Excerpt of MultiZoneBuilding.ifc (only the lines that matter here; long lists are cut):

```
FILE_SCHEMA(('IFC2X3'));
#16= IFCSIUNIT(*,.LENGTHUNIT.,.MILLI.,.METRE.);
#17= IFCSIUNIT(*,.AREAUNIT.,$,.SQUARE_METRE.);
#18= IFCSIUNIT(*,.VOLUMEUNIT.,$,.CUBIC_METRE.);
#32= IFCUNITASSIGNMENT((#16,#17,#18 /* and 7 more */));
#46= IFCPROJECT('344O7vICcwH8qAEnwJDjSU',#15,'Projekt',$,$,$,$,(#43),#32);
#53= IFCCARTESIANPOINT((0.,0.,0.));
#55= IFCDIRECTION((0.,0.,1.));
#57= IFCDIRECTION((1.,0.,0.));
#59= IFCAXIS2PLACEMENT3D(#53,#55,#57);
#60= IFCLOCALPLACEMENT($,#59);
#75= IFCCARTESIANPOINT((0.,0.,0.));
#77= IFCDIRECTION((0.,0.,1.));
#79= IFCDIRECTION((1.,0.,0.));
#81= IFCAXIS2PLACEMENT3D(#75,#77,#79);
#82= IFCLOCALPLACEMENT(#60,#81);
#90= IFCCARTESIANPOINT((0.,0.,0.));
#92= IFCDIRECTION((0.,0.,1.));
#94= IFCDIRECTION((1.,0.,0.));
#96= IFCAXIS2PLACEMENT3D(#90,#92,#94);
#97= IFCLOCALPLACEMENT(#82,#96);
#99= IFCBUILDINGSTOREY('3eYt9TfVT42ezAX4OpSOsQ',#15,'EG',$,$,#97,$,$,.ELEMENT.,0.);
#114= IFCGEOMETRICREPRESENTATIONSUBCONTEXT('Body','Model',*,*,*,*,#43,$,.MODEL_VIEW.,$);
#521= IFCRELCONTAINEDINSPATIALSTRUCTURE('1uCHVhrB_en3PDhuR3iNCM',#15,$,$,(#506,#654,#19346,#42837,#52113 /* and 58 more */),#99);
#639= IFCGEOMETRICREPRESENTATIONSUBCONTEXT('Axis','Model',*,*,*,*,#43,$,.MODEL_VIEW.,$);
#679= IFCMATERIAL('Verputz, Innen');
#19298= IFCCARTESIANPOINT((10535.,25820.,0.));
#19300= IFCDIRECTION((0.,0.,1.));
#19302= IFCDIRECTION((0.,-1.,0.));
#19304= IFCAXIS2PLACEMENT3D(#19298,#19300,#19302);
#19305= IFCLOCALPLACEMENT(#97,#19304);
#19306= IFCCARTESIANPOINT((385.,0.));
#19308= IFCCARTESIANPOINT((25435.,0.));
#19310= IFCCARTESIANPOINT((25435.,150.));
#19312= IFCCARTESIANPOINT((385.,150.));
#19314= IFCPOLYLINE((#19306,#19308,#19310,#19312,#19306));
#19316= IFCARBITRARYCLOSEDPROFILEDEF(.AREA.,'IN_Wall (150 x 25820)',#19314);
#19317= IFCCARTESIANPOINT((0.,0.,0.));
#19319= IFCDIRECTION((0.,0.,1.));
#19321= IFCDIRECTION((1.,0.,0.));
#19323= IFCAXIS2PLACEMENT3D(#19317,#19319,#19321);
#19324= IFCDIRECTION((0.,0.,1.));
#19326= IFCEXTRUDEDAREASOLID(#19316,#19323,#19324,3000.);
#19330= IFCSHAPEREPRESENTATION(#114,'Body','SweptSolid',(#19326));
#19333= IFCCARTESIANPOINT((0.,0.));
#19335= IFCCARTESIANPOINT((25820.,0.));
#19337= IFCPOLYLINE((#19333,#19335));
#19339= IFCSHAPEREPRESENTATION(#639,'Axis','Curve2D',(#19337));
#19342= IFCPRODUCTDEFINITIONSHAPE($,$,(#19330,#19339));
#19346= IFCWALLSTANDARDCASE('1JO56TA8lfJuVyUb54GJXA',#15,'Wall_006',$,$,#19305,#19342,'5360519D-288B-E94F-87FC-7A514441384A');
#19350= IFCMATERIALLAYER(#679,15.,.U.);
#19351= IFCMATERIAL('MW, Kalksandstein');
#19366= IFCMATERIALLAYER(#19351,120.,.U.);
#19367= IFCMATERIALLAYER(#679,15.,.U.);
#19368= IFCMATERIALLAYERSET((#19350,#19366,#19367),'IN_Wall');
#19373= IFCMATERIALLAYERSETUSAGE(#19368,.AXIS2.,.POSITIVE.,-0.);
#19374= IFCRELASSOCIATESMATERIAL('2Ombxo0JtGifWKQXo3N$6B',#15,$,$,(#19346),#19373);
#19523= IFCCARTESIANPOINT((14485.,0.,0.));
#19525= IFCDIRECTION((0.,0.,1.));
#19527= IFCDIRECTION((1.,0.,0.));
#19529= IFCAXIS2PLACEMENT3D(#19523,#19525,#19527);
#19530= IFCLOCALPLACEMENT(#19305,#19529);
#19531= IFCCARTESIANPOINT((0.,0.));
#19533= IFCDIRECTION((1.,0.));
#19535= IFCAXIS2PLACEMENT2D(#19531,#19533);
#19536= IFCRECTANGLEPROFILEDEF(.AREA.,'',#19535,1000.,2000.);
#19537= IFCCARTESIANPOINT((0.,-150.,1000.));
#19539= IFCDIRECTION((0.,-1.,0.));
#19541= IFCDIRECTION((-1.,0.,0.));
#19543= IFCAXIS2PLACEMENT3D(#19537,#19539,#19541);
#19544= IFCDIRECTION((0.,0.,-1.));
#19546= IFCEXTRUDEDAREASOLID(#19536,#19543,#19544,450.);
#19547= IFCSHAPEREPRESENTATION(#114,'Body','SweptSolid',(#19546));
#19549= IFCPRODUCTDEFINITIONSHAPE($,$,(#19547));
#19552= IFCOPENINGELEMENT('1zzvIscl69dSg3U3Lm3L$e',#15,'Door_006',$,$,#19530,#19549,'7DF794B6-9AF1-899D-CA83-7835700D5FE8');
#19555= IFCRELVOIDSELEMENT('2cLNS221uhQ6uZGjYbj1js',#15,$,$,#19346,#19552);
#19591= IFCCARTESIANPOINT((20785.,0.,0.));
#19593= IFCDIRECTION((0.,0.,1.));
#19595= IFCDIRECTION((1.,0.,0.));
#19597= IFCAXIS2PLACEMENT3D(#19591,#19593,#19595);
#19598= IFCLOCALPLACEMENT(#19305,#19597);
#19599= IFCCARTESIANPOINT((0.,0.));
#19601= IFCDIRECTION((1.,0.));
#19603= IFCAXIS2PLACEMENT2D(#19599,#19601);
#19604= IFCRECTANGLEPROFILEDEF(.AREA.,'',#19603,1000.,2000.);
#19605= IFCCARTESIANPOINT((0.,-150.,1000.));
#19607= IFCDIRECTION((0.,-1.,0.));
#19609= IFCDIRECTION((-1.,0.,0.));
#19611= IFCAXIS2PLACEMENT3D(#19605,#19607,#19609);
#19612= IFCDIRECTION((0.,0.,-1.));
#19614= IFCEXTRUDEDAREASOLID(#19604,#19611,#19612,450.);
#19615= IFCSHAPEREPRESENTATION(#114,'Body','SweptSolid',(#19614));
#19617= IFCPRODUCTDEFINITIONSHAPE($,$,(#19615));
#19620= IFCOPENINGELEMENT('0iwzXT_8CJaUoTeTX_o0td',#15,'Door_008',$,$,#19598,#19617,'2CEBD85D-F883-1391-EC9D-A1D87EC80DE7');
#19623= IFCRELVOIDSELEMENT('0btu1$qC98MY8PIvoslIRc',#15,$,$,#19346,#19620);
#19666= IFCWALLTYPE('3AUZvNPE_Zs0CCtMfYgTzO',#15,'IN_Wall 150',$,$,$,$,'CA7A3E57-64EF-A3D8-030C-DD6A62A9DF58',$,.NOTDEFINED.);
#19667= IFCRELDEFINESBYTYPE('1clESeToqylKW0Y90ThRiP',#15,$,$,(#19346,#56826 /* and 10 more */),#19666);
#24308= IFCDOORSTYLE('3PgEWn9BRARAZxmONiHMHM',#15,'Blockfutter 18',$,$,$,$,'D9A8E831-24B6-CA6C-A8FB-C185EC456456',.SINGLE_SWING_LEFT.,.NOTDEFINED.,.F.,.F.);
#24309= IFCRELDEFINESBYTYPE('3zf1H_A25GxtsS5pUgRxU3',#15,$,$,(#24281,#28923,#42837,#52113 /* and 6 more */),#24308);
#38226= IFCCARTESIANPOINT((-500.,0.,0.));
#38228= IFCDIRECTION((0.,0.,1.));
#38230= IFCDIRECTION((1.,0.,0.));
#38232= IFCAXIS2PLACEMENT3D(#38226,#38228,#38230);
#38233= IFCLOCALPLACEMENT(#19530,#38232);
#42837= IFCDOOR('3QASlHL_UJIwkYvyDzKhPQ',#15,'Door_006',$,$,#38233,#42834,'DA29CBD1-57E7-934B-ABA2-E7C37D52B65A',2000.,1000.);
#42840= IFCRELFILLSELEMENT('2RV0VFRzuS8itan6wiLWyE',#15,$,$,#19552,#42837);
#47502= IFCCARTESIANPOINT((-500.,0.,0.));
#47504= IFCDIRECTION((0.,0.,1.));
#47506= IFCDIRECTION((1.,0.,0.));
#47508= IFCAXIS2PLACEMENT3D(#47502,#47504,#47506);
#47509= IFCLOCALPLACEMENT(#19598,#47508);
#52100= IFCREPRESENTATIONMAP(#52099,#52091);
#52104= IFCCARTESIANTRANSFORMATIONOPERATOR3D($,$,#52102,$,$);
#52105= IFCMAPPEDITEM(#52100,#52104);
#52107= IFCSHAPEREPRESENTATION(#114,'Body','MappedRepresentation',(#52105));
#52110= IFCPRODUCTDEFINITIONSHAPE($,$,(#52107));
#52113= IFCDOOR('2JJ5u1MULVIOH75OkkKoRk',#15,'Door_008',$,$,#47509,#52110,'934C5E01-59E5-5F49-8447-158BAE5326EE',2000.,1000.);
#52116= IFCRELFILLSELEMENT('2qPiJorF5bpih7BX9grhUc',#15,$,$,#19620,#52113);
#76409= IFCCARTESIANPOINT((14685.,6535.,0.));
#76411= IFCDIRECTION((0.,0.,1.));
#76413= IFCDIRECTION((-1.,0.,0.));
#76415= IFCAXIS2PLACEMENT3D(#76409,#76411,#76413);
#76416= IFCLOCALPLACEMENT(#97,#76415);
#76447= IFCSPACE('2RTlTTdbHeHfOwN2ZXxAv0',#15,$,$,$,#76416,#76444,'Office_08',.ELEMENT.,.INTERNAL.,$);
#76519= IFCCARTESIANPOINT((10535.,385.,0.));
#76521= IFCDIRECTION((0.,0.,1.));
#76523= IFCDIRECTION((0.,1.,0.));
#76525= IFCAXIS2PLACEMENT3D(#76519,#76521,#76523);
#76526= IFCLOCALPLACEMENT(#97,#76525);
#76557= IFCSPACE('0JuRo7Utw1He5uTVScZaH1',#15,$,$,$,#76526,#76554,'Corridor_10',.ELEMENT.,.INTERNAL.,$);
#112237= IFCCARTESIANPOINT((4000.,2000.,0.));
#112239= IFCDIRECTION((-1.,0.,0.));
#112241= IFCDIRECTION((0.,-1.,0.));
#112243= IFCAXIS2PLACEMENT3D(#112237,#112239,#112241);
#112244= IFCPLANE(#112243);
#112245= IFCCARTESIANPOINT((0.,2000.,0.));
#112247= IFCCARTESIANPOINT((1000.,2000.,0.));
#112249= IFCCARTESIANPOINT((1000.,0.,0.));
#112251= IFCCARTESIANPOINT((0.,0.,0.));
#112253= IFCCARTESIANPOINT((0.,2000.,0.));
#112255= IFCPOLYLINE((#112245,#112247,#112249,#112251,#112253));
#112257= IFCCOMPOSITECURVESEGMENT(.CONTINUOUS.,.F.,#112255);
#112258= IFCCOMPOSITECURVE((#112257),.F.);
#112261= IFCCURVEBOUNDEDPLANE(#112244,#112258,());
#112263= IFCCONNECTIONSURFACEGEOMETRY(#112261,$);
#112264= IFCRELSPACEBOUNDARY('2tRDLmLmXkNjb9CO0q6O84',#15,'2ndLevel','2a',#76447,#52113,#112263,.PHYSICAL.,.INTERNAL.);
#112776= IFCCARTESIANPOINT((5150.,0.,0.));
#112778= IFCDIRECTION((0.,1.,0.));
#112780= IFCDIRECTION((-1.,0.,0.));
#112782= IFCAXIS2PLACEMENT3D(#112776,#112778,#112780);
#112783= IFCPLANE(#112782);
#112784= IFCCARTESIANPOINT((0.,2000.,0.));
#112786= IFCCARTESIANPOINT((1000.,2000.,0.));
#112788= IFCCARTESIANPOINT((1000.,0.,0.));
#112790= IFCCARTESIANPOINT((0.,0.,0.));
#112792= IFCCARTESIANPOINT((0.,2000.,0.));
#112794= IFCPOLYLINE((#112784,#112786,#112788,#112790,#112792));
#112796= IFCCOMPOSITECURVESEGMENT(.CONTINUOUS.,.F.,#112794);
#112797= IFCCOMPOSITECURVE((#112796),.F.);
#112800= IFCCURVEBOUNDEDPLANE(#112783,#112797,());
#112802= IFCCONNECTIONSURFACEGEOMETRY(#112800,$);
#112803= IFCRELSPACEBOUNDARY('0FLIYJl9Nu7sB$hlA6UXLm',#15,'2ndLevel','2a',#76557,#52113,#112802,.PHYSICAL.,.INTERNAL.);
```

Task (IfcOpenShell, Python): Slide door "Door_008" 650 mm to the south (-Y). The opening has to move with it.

```python
import numpy as np
import ifcopenshell
import ifcopenshell.api.geometry
import ifcopenshell.util.placement
import ifcopenshell.util.unit

model = ifcopenshell.open("MultiZoneBuilding.ifc")
unit_scale = ifcopenshell.util.unit.calculate_unit_scale(model)

door = model.by_guid("2JJ5u1MULVIOH75OkkKoRk")
opening = door.FillsVoids[0].RelatingOpeningElement
wall = opening.VoidsElements[0].RelatingBuildingElement

wall_matrix = ifcopenshell.util.placement.get_local_placement(wall.ObjectPlacement)
shift = wall_matrix[:3, 0] * 0.65 / unit_scale
before = ifcopenshell.util.placement.get_local_placement(door.ObjectPlacement)[:3, 3].copy()

# The door is placed relative to its opening, so it follows when the opening moves.
matrix = ifcopenshell.util.placement.get_local_placement(opening.ObjectPlacement)
matrix[:3, 3] += shift
ifcopenshell.api.geometry.edit_object_placement(
    model, product=opening, matrix=matrix, is_si=False, should_transform_children=True
)

# Space boundary surfaces are stored in each space's coordinates; move them too.
for rel in door.ProvidesBoundaries:
    if not rel.ConnectionGeometry:
        continue
    surface = rel.ConnectionGeometry.SurfaceOnRelatingElement.BasisSurface
    space_matrix = ifcopenshell.util.placement.get_local_placement(rel.RelatingSpace.ObjectPlacement)
    point = np.array(surface.Position.Location.Coordinates) + space_matrix[:3, :3].T @ shift
    surface.Position = model.createIfcAxis2Placement3D(
        model.createIfcCartesianPoint(point.tolist()), surface.Position.Axis, surface.Position.RefDirection
    )

after = ifcopenshell.util.placement.get_local_placement(door.ObjectPlacement)[:3, 3]
print("door moved by", (after - before).round(3) + 0.0)

model.write("MultiZoneBuilding_edited.ifc")
```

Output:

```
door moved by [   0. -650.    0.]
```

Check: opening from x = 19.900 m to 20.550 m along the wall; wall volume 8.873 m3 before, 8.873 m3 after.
